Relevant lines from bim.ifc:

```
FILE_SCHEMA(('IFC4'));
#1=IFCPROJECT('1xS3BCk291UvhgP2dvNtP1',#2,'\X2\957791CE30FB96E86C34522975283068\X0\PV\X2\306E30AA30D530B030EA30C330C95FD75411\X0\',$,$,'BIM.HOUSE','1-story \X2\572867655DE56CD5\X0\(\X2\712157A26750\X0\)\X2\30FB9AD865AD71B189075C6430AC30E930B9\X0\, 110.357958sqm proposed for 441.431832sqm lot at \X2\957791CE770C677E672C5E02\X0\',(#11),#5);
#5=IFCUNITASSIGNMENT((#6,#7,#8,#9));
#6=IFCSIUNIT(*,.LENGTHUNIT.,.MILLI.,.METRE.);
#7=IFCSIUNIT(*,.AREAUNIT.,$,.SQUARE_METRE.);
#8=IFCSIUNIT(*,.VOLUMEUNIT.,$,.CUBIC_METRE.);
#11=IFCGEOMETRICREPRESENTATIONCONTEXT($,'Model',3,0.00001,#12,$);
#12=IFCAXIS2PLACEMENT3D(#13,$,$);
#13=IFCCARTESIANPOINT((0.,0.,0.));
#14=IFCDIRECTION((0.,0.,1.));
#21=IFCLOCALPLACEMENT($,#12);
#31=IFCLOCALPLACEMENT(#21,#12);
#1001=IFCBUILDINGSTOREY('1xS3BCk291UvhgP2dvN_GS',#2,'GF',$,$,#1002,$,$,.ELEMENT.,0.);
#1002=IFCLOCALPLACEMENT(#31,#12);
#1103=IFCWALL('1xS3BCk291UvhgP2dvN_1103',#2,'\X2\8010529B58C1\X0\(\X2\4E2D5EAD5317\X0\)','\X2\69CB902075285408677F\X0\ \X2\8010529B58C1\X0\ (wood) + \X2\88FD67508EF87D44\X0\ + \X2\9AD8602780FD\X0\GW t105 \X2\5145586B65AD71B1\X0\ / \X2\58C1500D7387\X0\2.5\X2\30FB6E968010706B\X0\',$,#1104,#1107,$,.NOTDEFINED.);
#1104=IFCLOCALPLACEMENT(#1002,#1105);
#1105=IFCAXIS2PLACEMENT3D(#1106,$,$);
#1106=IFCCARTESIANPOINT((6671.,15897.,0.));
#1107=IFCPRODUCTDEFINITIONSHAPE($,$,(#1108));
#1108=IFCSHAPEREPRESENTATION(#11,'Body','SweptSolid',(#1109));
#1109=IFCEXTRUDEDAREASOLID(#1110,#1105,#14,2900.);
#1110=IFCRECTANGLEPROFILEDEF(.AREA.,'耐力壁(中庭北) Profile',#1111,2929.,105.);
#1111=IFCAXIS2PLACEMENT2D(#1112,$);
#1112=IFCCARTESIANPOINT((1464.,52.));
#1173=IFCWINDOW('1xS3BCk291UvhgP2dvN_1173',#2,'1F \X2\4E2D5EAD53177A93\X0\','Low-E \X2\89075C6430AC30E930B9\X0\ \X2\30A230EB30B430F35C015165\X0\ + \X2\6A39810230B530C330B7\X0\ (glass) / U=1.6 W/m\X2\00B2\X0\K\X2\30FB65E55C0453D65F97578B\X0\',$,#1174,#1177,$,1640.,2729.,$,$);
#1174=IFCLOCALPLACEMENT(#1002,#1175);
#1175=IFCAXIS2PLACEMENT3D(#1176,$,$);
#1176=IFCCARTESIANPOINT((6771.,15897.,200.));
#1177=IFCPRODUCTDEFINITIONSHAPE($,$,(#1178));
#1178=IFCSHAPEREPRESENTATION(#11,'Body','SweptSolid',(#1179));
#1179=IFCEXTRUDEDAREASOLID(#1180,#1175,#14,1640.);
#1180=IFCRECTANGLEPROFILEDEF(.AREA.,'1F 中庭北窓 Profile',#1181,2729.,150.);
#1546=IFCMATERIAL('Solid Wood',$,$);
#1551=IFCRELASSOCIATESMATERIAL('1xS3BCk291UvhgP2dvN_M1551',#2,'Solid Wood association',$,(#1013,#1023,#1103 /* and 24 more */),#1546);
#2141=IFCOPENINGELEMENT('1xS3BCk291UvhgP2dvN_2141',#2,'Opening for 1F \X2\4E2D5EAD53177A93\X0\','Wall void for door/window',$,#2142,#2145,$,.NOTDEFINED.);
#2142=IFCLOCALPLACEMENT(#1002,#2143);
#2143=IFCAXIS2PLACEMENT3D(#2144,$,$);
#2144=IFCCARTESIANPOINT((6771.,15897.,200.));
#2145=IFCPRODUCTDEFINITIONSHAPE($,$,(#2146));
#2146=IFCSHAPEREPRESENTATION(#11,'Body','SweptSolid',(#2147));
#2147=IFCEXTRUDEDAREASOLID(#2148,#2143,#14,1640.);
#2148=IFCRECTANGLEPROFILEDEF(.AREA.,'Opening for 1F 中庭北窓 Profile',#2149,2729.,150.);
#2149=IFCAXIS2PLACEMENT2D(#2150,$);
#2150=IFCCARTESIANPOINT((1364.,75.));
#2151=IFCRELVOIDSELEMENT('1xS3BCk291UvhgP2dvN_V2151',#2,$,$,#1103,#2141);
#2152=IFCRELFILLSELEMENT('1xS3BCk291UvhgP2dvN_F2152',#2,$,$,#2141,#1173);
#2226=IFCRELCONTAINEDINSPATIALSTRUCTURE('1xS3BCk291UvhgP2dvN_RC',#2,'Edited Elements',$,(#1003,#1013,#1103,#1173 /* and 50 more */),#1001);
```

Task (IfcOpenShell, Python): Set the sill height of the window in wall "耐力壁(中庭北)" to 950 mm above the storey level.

```python
import numpy as np
import ifcopenshell
import ifcopenshell.api.geometry
import ifcopenshell.geom
import ifcopenshell.util.element
import ifcopenshell.util.placement
import ifcopenshell.util.shape
import ifcopenshell.util.unit

model = ifcopenshell.open("bim.ifc")
unit_scale = ifcopenshell.util.unit.calculate_unit_scale(model)

window = model.by_guid("1xS3BCk291UvhgP2dvN_1173")
opening = window.FillsVoids[0].RelatingOpeningElement
storey = ifcopenshell.util.element.get_container(window, ifc_class="IfcBuildingStorey")
level = ifcopenshell.util.placement.get_local_placement(storey.ObjectPlacement)[2, 3]

# The opening's origin need not be at the sill, so measure its lowest point.
shape = ifcopenshell.geom.create_shape(ifcopenshell.geom.settings(), opening)
bottom = ifcopenshell.util.shape.get_shape_bottom_elevation(shape, shape.geometry) / unit_scale
dz = level + 0.95 / unit_scale - bottom

shift = np.array([0.0, 0.0, dz])
# The window is not placed relative to its opening, so move both.
for product in (opening, window):
    matrix = ifcopenshell.util.placement.get_local_placement(product.ObjectPlacement)
    matrix[:3, 3] += shift
    ifcopenshell.api.geometry.edit_object_placement(model, product=product, matrix=matrix, is_si=False)

print(f"moved by {dz * unit_scale:+.3f} m")

model.write("bim_v2.ifc")
```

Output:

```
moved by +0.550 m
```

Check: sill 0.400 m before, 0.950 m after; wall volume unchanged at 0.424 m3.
